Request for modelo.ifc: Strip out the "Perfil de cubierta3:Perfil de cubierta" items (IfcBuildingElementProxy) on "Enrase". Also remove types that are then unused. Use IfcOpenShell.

First a look at what the model holds.

```python
import ifcopenshell
import ifcopenshell.util.element

model = ifcopenshell.open("modelo.ifc")
print(model.schema)
storey = next(s for s in model.by_type("IfcBuildingStorey") if s.Name == "Enrase")
proxies = [e for e in ifcopenshell.util.element.get_decomposition(storey) if e.is_a("IfcBuildingElementProxy")]
seen = {}
for e in proxies:
    element_type = ifcopenshell.util.element.get_type(e)
    name = element_type.Name if element_type not in (None, e) else None
    seen[name] = seen.get(name, 0) + 1
for name, count in sorted(seen.items(), key=str):
    print(count, "x", name)
```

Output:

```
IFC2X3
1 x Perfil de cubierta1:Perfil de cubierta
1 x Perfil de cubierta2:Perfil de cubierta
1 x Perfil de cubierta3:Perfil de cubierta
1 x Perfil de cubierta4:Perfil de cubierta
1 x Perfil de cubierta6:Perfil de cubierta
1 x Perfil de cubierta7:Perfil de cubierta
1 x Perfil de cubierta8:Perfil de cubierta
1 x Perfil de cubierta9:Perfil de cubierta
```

```python
import ifcopenshell
import ifcopenshell.api.root
import ifcopenshell.util.element

model = ifcopenshell.open("modelo.ifc")

storey = next(s for s in model.by_type("IfcBuildingStorey") if s.Name == "Enrase")
proxies = [e for e in ifcopenshell.util.element.get_decomposition(storey) if e.is_a("IfcBuildingElementProxy")]
targets = [e for e in proxies if (t := ifcopenshell.util.element.get_type(e)) not in (None, e) and t.Name == "Perfil de cubierta3:Perfil de cubierta"]
types = {ifcopenshell.util.element.get_type(e) for e in targets} - {None, *targets}

for e in targets:
    ifcopenshell.api.root.remove_product(model, product=e)
print(len(targets), "removed")

unused = [t for t in types if not ifcopenshell.util.element.get_types(t)]
for t in unused:
    ifcopenshell.api.root.remove_product(model, product=t)
print(len(unused), "unused types removed")

model.write("modelo-out.ifc")
```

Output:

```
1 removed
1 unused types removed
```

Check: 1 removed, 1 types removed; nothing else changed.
